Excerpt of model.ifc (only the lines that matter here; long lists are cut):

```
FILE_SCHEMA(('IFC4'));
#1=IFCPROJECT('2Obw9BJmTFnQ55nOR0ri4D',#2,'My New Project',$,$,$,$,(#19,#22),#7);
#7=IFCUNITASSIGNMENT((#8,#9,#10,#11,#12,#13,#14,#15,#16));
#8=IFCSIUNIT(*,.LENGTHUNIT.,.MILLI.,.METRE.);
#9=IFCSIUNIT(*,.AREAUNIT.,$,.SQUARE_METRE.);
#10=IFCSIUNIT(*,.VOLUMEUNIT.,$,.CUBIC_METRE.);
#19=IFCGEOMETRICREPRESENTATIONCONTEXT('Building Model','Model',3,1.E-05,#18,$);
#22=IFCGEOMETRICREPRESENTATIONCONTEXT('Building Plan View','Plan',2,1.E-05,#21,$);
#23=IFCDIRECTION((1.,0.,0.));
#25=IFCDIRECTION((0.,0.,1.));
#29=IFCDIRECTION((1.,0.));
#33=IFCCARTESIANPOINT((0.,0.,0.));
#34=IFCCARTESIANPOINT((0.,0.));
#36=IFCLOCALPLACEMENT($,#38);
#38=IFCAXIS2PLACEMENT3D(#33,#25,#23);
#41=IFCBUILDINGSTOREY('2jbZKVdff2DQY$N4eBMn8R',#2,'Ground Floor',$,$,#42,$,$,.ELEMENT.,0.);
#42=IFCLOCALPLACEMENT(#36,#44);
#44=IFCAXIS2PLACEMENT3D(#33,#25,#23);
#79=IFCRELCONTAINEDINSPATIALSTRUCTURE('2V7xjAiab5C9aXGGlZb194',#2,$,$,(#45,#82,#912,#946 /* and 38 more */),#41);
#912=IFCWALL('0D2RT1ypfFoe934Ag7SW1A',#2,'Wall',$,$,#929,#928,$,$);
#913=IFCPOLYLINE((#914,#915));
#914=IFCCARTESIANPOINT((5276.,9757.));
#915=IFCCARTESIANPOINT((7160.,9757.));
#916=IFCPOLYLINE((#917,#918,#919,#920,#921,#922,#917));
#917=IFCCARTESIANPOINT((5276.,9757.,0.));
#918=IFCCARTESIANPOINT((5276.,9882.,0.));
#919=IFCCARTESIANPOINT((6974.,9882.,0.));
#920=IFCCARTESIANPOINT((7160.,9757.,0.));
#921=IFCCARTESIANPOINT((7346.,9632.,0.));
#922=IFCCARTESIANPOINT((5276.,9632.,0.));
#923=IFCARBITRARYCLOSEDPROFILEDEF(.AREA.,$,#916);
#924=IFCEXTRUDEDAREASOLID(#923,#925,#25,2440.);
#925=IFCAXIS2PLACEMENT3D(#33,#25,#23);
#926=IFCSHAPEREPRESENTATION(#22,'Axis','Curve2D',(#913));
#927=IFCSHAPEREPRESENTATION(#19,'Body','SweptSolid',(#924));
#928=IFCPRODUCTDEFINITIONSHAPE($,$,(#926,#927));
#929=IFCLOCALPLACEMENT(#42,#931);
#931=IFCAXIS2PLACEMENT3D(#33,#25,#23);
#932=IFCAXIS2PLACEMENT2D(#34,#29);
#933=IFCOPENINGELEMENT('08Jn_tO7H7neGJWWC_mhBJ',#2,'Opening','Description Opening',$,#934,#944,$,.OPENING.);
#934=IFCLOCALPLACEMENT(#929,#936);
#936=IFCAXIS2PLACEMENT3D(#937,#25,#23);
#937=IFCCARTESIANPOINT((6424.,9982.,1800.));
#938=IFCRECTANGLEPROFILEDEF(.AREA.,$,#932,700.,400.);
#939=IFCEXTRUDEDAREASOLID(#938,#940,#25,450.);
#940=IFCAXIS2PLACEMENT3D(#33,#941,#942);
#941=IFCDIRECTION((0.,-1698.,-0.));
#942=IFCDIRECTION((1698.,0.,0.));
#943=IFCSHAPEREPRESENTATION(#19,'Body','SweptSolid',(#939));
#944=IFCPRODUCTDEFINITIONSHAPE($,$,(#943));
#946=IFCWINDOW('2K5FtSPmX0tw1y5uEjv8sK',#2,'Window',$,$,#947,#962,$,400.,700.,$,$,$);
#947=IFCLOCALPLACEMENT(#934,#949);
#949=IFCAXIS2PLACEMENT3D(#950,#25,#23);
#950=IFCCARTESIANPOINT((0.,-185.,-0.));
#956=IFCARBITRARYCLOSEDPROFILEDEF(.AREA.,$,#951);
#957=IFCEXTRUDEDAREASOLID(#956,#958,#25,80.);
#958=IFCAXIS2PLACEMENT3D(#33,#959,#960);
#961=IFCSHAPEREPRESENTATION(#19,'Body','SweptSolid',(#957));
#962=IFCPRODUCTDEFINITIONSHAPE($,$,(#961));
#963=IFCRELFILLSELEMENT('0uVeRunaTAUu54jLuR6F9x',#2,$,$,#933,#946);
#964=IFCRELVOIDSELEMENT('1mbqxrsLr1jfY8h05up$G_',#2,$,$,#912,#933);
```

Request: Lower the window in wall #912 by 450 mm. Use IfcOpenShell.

```python
import numpy as np
import ifcopenshell
import ifcopenshell.api.geometry
import ifcopenshell.util.placement
import ifcopenshell.util.unit

model = ifcopenshell.open("model.ifc")
unit_scale = ifcopenshell.util.unit.calculate_unit_scale(model)

window = model.by_id(946)
opening = window.FillsVoids[0].RelatingOpeningElement
dz = -450.0

shift = np.array([0.0, 0.0, dz])
# The window is placed relative to its opening, so it follows when the opening moves.
matrix = ifcopenshell.util.placement.get_local_placement(opening.ObjectPlacement)
matrix[:3, 3] += shift
ifcopenshell.api.geometry.edit_object_placement(
    model, product=opening, matrix=matrix, is_si=False, should_transform_children=True
)

print(f"moved by {dz * unit_scale:+.3f} m")

model.write("model_rev.ifc")
```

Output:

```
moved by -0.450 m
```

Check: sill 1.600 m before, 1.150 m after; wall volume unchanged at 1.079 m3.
